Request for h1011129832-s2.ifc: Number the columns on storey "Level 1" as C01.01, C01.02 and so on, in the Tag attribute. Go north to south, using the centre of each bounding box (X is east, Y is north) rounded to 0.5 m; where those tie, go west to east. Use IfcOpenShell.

First a look at what the model holds.

```python
import ifcopenshell
import ifcopenshell.util.element
import ifcopenshell.util.placement

model = ifcopenshell.open("h1011129832-s2.ifc")
print(model.schema)
storey = next(s for s in model.by_type("IfcBuildingStorey") if s.Name == "Level 1")
columns = [e for e in ifcopenshell.util.element.get_decomposition(storey) if e.is_a("IfcColumn")]
for e in sorted(columns, key=lambda e: e.id()):
    origin = ifcopenshell.util.placement.get_local_placement(e.ObjectPlacement)[:3, 3]
    print(e.id(), e.Tag, e.Name, origin.round(2) + 0.0, sep=" | ")
```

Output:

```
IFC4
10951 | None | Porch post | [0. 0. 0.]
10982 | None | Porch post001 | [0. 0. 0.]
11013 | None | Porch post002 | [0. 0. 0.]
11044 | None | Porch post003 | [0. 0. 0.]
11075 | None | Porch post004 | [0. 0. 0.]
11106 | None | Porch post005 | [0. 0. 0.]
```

```python
import ifcopenshell
import ifcopenshell.geom
import ifcopenshell.util.element
import ifcopenshell.util.shape

model = ifcopenshell.open("h1011129832-s2.ifc")
settings = ifcopenshell.geom.settings()
settings.set("use-world-coords", True)


def centre(element):
    shape = ifcopenshell.geom.create_shape(settings, element)
    return ifcopenshell.util.shape.get_bbox_centroid(shape.geometry)


storey = next(s for s in model.by_type("IfcBuildingStorey") if s.Name == "Level 1")
columns = [e for e in ifcopenshell.util.element.get_decomposition(storey) if e.is_a("IfcColumn")]

# Insertion points can sit at a corner or the storey origin, so sort by the geometry (in metres).
centres = {e: centre(e) for e in columns}
columns.sort(key=lambda e: (-round(centres[e][1] / 0.5), centres[e][0]))

for i, e in enumerate(columns, start=1):
    number = f"C01.{i:02d}"
    e.Tag = number
    print(e.id(), number)

model.write("h1011129832-s2_edited.ifc")
```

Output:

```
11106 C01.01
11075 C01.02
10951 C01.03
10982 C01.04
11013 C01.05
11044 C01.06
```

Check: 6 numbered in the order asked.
